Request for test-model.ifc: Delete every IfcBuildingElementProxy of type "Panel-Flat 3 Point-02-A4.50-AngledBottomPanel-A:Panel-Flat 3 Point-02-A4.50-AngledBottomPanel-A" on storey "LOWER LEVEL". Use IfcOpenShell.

First a look at what the model holds.

```python
import ifcopenshell
import ifcopenshell.util.element

model = ifcopenshell.open("test-model.ifc")
print(model.schema)
storey = next(s for s in model.by_type("IfcBuildingStorey") if s.Name == "LOWER LEVEL")
proxies = [e for e in ifcopenshell.util.element.get_decomposition(storey) if e.is_a("IfcBuildingElementProxy")]
seen = {}
for e in proxies:
    element_type = ifcopenshell.util.element.get_type(e)
    name = element_type.Name if element_type not in (None, e) else None
    seen[name] = seen.get(name, 0) + 1
for name, count in sorted(seen.items(), key=str):
    print(count, "x", name)
```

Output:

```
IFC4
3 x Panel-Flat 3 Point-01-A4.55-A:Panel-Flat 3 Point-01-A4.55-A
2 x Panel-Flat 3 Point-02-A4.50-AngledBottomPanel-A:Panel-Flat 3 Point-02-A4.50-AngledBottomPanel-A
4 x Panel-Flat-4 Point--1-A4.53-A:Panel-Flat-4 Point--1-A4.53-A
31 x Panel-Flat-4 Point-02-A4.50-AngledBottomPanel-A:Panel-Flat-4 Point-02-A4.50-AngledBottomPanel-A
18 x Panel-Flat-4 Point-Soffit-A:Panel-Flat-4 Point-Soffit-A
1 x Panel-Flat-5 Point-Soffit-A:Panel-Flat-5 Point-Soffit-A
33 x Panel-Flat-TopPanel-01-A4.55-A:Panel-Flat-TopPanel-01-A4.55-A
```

```python
import ifcopenshell
import ifcopenshell.api.root
import ifcopenshell.util.element

model = ifcopenshell.open("test-model.ifc")

storey = next(s for s in model.by_type("IfcBuildingStorey") if s.Name == "LOWER LEVEL")
proxies = [e for e in ifcopenshell.util.element.get_decomposition(storey) if e.is_a("IfcBuildingElementProxy")]
targets = [e for e in proxies if (t := ifcopenshell.util.element.get_type(e)) not in (None, e) and t.Name == "Panel-Flat 3 Point-02-A4.50-AngledBottomPanel-A:Panel-Flat 3 Point-02-A4.50-AngledBottomPanel-A"]

for e in targets:
    ifcopenshell.api.root.remove_product(model, product=e)
print(len(targets), "removed")

model.write("test-model_v2.ifc")
```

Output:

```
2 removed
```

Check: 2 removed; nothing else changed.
